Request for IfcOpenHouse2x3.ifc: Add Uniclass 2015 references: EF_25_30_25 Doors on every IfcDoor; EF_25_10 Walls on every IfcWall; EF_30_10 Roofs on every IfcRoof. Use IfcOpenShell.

First a look at what the model holds.

```python
import ifcopenshell

model = ifcopenshell.open("IfcOpenHouse2x3.ifc")
print(model.schema)
print("classifications:", [c.Name for c in model.by_type("IfcClassification")])
for ifc_class in ("IfcDoor", "IfcRoof", "IfcStair", "IfcWall", "IfcWindow"):
    print(ifc_class, len(model.by_type(ifc_class)))
```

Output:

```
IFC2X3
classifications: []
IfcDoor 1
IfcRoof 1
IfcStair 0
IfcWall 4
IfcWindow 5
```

```python
import ifcopenshell
import ifcopenshell.api.classification

model = ifcopenshell.open("IfcOpenHouse2x3.ifc")

# IFC2X3 requires Source and Edition and has no link from the project to the system.
system = model.create_entity("IfcClassification", Source="NBS", Edition="2015", Name="Uniclass 2015")

codes = {
    "IfcDoor": ("EF_25_30_25", "Doors"),
    "IfcWall": ("EF_25_10", "Walls"),
    "IfcRoof": ("EF_30_10", "Roofs"),
}
for ifc_class, (code, name) in codes.items():
    products = model.by_type(ifc_class)
    ifcopenshell.api.classification.add_reference(
        model, products=products, classification=system, identification=code, name=name
    )
    print(code, len(products))

model.write("IfcOpenHouse2x3_v2.ifc")
```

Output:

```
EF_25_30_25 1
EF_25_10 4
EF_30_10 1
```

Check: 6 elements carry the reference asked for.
